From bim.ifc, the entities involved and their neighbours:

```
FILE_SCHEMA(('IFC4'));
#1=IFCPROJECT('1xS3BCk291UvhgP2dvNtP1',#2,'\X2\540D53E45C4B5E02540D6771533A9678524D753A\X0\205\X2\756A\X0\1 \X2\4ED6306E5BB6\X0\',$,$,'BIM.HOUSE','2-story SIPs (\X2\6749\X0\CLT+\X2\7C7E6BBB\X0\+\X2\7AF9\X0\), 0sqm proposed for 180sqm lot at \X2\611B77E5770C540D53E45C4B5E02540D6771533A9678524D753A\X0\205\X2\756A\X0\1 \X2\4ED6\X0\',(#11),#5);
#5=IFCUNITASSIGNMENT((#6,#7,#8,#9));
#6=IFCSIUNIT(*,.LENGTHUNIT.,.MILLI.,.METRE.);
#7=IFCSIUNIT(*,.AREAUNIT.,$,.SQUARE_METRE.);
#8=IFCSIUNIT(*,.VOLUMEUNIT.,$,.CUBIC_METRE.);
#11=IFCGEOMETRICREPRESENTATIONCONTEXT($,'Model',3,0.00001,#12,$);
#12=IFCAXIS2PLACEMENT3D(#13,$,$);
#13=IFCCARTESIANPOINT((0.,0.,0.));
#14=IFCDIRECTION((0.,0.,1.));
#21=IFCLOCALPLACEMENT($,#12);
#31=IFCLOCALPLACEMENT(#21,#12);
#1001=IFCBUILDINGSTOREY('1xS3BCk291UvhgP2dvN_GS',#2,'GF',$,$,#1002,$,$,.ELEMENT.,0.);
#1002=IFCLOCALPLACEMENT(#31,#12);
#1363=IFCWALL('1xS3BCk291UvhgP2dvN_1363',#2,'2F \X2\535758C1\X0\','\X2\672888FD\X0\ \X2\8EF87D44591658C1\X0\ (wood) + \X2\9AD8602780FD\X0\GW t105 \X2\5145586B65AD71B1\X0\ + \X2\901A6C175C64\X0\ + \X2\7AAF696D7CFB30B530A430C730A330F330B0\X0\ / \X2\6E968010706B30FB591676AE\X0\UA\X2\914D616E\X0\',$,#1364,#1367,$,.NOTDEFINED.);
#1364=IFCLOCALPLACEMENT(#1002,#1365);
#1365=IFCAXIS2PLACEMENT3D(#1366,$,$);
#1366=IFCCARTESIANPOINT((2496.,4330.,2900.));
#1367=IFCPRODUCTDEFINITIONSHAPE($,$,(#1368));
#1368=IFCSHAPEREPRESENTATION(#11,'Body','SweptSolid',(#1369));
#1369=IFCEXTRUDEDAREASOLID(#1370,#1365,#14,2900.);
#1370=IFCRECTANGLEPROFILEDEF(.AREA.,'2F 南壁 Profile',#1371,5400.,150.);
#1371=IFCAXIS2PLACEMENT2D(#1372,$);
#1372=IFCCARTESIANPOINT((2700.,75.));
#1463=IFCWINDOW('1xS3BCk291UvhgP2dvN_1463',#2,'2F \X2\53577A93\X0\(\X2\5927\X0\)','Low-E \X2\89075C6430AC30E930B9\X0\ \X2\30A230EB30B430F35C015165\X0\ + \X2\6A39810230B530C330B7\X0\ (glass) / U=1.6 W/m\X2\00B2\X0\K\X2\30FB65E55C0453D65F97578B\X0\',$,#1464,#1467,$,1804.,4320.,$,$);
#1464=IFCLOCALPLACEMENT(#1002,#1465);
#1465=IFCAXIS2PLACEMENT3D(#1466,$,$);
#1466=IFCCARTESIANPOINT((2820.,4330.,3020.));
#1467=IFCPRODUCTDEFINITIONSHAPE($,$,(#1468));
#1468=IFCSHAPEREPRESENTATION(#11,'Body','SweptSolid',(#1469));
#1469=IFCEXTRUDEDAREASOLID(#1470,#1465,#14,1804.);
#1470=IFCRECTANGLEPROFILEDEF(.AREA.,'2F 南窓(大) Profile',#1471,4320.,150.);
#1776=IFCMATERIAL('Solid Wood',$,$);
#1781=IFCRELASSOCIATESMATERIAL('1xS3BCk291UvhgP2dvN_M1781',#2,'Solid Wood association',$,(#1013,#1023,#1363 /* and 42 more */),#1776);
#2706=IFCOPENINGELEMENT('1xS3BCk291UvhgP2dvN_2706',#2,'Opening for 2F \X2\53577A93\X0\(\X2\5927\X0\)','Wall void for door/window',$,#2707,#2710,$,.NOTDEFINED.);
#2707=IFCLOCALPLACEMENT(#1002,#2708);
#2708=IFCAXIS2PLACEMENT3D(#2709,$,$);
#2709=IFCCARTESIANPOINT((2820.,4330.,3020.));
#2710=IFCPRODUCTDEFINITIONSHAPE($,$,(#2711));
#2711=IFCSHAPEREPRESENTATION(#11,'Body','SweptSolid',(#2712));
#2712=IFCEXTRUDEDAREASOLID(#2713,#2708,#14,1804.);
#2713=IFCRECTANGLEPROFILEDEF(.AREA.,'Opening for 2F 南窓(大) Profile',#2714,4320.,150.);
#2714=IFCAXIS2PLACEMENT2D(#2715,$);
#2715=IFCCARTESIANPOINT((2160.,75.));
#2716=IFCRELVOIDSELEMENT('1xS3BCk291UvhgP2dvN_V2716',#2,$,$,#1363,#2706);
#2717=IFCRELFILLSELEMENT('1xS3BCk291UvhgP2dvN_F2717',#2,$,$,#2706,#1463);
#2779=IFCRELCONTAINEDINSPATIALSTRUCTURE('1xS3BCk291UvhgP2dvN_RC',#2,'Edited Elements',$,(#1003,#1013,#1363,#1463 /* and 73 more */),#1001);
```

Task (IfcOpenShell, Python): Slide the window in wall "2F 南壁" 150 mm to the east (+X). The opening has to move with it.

```python
import ifcopenshell
import ifcopenshell.api.geometry
import ifcopenshell.util.placement

model = ifcopenshell.open("bim.ifc")

window = model.by_guid("1xS3BCk291UvhgP2dvN_1463")
opening = window.FillsVoids[0].RelatingOpeningElement
wall = opening.VoidsElements[0].RelatingBuildingElement

wall_matrix = ifcopenshell.util.placement.get_local_placement(wall.ObjectPlacement)
shift = wall_matrix[:3, 0] * 150.0
before = ifcopenshell.util.placement.get_local_placement(window.ObjectPlacement)[:3, 3].copy()

# The window is not placed relative to its opening, so move both.
for product in (opening, window):
    matrix = ifcopenshell.util.placement.get_local_placement(product.ObjectPlacement)
    matrix[:3, 3] += shift
    ifcopenshell.api.geometry.edit_object_placement(model, product=product, matrix=matrix, is_si=False)

after = ifcopenshell.util.placement.get_local_placement(window.ObjectPlacement)[:3, 3]
print("window moved by", (after - before).round(3) + 0.0)

model.write("bim_rev.ifc")
```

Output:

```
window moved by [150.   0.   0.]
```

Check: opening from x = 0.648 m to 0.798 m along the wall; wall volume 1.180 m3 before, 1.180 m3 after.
